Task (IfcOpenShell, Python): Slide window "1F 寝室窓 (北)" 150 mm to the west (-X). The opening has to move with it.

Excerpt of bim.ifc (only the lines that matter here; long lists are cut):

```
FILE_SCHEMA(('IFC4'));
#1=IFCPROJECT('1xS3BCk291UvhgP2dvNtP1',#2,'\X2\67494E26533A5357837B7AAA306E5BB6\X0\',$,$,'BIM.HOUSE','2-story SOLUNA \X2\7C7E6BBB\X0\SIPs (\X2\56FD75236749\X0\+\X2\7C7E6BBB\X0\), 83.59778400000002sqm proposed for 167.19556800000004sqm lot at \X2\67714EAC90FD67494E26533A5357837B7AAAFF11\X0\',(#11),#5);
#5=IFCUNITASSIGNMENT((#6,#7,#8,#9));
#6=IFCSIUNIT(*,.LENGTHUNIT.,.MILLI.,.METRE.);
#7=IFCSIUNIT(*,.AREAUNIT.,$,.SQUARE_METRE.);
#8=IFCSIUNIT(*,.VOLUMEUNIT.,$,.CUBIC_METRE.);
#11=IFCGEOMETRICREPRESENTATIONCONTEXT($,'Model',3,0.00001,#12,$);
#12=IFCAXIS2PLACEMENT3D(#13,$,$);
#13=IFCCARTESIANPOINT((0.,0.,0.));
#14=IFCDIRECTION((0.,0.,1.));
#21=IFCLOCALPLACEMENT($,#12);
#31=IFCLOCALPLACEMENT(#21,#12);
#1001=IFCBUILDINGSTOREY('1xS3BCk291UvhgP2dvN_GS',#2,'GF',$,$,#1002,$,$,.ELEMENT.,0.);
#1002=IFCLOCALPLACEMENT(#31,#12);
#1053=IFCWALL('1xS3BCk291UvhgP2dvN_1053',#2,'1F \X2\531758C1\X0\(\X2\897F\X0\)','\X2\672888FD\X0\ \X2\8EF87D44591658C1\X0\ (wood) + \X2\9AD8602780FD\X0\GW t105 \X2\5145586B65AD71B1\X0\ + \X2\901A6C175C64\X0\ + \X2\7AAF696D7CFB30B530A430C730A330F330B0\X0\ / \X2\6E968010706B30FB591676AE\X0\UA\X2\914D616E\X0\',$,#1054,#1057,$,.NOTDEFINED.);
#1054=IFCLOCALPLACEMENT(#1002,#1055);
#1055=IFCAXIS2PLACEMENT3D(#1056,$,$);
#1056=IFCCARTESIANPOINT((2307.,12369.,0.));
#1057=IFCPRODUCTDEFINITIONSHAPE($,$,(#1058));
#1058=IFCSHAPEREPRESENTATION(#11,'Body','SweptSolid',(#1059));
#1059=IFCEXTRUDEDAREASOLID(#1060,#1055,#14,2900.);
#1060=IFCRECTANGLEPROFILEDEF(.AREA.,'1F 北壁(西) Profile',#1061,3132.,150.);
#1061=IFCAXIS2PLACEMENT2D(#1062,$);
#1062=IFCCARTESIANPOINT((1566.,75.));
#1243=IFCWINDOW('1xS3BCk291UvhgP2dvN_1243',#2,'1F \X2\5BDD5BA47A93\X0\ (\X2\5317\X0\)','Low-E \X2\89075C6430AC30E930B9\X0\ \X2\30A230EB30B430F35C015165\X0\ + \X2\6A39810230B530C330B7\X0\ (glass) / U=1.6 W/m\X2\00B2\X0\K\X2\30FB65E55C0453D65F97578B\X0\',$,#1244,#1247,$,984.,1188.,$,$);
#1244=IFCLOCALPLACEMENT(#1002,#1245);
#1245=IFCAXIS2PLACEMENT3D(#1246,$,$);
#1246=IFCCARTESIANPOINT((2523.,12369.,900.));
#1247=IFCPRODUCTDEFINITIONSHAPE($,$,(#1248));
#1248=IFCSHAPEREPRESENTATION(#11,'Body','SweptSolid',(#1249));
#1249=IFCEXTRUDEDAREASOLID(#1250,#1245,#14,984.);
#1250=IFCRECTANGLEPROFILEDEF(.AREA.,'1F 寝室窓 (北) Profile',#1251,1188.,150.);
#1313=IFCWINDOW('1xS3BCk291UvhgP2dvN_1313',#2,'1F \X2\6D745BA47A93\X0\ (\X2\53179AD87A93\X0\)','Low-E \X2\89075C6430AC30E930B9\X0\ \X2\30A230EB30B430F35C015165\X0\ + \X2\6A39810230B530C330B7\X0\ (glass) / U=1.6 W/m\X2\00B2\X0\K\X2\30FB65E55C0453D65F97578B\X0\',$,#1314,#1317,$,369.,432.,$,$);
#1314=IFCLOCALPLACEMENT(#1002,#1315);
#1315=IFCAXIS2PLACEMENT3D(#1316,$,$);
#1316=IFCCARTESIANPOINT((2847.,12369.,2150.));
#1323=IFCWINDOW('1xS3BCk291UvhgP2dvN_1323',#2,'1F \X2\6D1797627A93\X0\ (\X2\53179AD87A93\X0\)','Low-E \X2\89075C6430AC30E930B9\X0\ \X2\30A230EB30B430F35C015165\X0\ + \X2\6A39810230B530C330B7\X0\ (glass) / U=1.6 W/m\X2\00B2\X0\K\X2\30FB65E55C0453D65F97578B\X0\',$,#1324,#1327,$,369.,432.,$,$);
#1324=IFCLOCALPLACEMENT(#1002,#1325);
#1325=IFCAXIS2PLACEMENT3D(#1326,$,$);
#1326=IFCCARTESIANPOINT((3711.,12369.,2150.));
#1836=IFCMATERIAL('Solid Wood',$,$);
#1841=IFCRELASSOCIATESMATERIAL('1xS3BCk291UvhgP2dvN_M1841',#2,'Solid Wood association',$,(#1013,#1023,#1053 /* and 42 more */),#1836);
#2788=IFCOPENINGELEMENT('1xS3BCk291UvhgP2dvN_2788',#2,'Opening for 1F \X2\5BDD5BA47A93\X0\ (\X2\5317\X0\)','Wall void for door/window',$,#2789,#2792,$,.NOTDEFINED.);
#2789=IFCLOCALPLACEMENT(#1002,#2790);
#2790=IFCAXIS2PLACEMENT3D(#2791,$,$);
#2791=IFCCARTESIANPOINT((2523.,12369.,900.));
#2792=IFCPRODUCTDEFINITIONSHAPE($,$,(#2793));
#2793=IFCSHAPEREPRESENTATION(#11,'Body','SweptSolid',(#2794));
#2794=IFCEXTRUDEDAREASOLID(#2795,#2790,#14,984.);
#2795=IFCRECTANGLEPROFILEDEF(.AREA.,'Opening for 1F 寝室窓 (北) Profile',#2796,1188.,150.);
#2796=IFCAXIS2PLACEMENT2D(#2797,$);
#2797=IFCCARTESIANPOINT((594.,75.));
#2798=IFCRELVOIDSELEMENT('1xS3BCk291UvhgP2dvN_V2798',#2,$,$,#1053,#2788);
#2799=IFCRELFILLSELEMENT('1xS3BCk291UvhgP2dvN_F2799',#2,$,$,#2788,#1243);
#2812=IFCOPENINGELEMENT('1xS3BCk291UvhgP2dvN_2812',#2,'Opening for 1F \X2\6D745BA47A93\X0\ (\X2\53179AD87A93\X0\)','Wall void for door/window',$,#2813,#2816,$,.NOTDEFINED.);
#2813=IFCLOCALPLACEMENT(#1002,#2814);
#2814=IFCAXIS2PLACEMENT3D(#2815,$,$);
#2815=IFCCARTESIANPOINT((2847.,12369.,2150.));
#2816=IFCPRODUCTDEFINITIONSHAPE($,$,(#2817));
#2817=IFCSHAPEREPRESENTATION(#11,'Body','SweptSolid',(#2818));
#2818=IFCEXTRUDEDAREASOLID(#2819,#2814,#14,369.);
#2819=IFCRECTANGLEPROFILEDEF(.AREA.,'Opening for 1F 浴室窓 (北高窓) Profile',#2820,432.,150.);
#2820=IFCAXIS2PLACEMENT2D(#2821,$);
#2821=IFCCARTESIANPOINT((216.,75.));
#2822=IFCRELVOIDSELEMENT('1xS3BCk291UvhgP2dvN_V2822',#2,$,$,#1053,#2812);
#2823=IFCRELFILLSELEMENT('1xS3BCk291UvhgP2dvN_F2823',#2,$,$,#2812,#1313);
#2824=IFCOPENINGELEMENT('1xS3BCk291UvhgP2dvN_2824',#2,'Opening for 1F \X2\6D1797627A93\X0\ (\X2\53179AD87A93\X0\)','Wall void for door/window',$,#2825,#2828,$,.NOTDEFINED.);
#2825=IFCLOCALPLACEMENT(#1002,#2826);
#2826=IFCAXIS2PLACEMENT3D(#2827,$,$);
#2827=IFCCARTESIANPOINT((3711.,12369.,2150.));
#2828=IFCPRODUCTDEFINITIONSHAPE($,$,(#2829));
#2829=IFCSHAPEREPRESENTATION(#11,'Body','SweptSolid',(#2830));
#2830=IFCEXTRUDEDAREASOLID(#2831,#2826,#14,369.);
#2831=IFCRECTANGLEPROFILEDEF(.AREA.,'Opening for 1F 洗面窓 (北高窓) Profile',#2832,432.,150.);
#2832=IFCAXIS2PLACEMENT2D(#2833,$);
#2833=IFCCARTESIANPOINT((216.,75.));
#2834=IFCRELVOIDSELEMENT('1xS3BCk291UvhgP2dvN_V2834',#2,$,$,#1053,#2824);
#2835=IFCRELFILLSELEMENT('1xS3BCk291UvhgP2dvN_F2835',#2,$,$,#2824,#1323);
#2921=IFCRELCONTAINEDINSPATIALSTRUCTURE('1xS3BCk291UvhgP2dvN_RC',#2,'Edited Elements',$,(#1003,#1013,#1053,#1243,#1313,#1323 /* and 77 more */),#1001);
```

```python
import ifcopenshell
import ifcopenshell.api.geometry
import ifcopenshell.util.placement
import ifcopenshell.util.unit

model = ifcopenshell.open("bim.ifc")
unit_scale = ifcopenshell.util.unit.calculate_unit_scale(model)

window = model.by_id(1243)
opening = window.FillsVoids[0].RelatingOpeningElement
wall = opening.VoidsElements[0].RelatingBuildingElement

wall_matrix = ifcopenshell.util.placement.get_local_placement(wall.ObjectPlacement)
shift = wall_matrix[:3, 0] * -0.15 / unit_scale
before = ifcopenshell.util.placement.get_local_placement(window.ObjectPlacement)[:3, 3].copy()

# The window is not placed relative to its opening, so move both.
for product in (opening, window):
    matrix = ifcopenshell.util.placement.get_local_placement(product.ObjectPlacement)
    matrix[:3, 3] += shift
    ifcopenshell.api.geometry.edit_object_placement(model, product=product, matrix=matrix, is_si=False)

after = ifcopenshell.util.placement.get_local_placement(window.ObjectPlacement)[:3, 3]
print("window moved by", (after - before).round(3) + 0.0)

model.write("bim_updated.ifc")
```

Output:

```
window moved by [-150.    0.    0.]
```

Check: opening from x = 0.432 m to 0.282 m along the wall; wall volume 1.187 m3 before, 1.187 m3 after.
